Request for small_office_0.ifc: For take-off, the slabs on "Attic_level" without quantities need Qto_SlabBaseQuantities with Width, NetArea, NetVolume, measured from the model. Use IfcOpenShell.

First a look at what the model holds.

```python
import ifcopenshell
import ifcopenshell.util.element
import ifcopenshell.util.unit

model = ifcopenshell.open("small_office_0.ifc")
print(model.schema)
for unit_type in ("LENGTHUNIT", "AREAUNIT", "VOLUMEUNIT"):
    print(unit_type, ifcopenshell.util.unit.calculate_unit_scale(model, unit_type))
storey = next(s for s in model.by_type("IfcBuildingStorey") if s.Name == "Attic_level")
slabs = [e for e in ifcopenshell.util.element.get_decomposition(storey) if e.is_a("IfcSlab")]
for e in sorted(slabs, key=lambda e: e.id()):
    print(e.id(), e.is_a(), e.Name, list(ifcopenshell.util.element.get_psets(e, qtos_only=True)), sep=" | ")
```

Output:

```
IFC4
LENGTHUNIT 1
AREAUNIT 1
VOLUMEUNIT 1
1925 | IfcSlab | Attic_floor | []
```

```python
import ifcopenshell
import ifcopenshell.api.pset
import ifcopenshell.geom
import ifcopenshell.util.element
import ifcopenshell.util.shape
import ifcopenshell.util.unit

model = ifcopenshell.open("small_office_0.ifc")
unit_scale = ifcopenshell.util.unit.calculate_unit_scale(model)
area_scale = ifcopenshell.util.unit.calculate_unit_scale(model, "AREAUNIT")
volume_scale = ifcopenshell.util.unit.calculate_unit_scale(model, "VOLUMEUNIT")
settings = ifcopenshell.geom.settings()

storey = next(s for s in model.by_type("IfcBuildingStorey") if s.Name == "Attic_level")
slabs = [e for e in ifcopenshell.util.element.get_decomposition(storey) if e.is_a("IfcSlab")]

for e in sorted(slabs, key=lambda e: e.id()):
    if ifcopenshell.util.element.get_psets(e, qtos_only=True, should_inherit=False):
        continue
    # Geometry comes back in metres, in the element's own axes.
    shape = ifcopenshell.geom.create_shape(settings, e)
    values = {
        "Width": ifcopenshell.util.shape.get_z(shape.geometry) / unit_scale,
        "NetArea": ifcopenshell.util.shape.get_footprint_area(shape.geometry) / area_scale,
        "NetVolume": ifcopenshell.util.shape.get_volume(shape.geometry) / volume_scale,
    }
    qto = ifcopenshell.api.pset.add_qto(model, product=e, name="Qto_SlabBaseQuantities")
    ifcopenshell.api.pset.edit_qto(model, qto=qto, properties=values)
    print(e.id(), {k: round(v, 3) for k, v in values.items()})

model.write("small_office_0_edited.ifc")
```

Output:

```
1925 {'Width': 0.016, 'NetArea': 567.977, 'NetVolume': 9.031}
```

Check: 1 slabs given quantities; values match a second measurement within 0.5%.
